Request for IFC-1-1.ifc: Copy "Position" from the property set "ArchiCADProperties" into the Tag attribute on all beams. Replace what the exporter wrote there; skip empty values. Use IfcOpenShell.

First a look at what the model holds.

```python
import ifcopenshell
import ifcopenshell.util.element

model = ifcopenshell.open("IFC-1-1.ifc")
print(model.schema)
beams = model.by_type("IfcBeam")
print(len(beams), "beams")
for e in beams[:8]:
    source = ifcopenshell.util.element.get_pset(e, "ArchiCADProperties", "Position")
    target = e.Tag
    print(e.id(), repr(source), repr(target), sep=" | ")
```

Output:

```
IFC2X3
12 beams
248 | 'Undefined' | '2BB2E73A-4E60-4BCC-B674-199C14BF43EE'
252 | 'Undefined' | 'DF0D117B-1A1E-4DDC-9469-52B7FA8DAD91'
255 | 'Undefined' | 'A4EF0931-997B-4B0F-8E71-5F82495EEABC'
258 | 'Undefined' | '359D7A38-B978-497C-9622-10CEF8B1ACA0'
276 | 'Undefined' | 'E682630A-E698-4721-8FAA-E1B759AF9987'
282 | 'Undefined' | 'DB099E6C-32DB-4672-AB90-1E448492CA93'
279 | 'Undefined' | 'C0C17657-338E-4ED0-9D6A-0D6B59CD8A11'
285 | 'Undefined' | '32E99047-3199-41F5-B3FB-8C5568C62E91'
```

```python
import ifcopenshell
import ifcopenshell.util.element

model = ifcopenshell.open("IFC-1-1.ifc")

count = 0
for e in model.by_type("IfcBeam"):
    value = ifcopenshell.util.element.get_pset(e, "ArchiCADProperties", "Position")
    current = e.Tag
    if not value or not value.strip() or current == value:
        continue
    e.Tag = value
    count += 1

print(count, "beams updated")

model.write("IFC-1-1_v2.ifc")
```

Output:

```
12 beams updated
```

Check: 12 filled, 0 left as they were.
